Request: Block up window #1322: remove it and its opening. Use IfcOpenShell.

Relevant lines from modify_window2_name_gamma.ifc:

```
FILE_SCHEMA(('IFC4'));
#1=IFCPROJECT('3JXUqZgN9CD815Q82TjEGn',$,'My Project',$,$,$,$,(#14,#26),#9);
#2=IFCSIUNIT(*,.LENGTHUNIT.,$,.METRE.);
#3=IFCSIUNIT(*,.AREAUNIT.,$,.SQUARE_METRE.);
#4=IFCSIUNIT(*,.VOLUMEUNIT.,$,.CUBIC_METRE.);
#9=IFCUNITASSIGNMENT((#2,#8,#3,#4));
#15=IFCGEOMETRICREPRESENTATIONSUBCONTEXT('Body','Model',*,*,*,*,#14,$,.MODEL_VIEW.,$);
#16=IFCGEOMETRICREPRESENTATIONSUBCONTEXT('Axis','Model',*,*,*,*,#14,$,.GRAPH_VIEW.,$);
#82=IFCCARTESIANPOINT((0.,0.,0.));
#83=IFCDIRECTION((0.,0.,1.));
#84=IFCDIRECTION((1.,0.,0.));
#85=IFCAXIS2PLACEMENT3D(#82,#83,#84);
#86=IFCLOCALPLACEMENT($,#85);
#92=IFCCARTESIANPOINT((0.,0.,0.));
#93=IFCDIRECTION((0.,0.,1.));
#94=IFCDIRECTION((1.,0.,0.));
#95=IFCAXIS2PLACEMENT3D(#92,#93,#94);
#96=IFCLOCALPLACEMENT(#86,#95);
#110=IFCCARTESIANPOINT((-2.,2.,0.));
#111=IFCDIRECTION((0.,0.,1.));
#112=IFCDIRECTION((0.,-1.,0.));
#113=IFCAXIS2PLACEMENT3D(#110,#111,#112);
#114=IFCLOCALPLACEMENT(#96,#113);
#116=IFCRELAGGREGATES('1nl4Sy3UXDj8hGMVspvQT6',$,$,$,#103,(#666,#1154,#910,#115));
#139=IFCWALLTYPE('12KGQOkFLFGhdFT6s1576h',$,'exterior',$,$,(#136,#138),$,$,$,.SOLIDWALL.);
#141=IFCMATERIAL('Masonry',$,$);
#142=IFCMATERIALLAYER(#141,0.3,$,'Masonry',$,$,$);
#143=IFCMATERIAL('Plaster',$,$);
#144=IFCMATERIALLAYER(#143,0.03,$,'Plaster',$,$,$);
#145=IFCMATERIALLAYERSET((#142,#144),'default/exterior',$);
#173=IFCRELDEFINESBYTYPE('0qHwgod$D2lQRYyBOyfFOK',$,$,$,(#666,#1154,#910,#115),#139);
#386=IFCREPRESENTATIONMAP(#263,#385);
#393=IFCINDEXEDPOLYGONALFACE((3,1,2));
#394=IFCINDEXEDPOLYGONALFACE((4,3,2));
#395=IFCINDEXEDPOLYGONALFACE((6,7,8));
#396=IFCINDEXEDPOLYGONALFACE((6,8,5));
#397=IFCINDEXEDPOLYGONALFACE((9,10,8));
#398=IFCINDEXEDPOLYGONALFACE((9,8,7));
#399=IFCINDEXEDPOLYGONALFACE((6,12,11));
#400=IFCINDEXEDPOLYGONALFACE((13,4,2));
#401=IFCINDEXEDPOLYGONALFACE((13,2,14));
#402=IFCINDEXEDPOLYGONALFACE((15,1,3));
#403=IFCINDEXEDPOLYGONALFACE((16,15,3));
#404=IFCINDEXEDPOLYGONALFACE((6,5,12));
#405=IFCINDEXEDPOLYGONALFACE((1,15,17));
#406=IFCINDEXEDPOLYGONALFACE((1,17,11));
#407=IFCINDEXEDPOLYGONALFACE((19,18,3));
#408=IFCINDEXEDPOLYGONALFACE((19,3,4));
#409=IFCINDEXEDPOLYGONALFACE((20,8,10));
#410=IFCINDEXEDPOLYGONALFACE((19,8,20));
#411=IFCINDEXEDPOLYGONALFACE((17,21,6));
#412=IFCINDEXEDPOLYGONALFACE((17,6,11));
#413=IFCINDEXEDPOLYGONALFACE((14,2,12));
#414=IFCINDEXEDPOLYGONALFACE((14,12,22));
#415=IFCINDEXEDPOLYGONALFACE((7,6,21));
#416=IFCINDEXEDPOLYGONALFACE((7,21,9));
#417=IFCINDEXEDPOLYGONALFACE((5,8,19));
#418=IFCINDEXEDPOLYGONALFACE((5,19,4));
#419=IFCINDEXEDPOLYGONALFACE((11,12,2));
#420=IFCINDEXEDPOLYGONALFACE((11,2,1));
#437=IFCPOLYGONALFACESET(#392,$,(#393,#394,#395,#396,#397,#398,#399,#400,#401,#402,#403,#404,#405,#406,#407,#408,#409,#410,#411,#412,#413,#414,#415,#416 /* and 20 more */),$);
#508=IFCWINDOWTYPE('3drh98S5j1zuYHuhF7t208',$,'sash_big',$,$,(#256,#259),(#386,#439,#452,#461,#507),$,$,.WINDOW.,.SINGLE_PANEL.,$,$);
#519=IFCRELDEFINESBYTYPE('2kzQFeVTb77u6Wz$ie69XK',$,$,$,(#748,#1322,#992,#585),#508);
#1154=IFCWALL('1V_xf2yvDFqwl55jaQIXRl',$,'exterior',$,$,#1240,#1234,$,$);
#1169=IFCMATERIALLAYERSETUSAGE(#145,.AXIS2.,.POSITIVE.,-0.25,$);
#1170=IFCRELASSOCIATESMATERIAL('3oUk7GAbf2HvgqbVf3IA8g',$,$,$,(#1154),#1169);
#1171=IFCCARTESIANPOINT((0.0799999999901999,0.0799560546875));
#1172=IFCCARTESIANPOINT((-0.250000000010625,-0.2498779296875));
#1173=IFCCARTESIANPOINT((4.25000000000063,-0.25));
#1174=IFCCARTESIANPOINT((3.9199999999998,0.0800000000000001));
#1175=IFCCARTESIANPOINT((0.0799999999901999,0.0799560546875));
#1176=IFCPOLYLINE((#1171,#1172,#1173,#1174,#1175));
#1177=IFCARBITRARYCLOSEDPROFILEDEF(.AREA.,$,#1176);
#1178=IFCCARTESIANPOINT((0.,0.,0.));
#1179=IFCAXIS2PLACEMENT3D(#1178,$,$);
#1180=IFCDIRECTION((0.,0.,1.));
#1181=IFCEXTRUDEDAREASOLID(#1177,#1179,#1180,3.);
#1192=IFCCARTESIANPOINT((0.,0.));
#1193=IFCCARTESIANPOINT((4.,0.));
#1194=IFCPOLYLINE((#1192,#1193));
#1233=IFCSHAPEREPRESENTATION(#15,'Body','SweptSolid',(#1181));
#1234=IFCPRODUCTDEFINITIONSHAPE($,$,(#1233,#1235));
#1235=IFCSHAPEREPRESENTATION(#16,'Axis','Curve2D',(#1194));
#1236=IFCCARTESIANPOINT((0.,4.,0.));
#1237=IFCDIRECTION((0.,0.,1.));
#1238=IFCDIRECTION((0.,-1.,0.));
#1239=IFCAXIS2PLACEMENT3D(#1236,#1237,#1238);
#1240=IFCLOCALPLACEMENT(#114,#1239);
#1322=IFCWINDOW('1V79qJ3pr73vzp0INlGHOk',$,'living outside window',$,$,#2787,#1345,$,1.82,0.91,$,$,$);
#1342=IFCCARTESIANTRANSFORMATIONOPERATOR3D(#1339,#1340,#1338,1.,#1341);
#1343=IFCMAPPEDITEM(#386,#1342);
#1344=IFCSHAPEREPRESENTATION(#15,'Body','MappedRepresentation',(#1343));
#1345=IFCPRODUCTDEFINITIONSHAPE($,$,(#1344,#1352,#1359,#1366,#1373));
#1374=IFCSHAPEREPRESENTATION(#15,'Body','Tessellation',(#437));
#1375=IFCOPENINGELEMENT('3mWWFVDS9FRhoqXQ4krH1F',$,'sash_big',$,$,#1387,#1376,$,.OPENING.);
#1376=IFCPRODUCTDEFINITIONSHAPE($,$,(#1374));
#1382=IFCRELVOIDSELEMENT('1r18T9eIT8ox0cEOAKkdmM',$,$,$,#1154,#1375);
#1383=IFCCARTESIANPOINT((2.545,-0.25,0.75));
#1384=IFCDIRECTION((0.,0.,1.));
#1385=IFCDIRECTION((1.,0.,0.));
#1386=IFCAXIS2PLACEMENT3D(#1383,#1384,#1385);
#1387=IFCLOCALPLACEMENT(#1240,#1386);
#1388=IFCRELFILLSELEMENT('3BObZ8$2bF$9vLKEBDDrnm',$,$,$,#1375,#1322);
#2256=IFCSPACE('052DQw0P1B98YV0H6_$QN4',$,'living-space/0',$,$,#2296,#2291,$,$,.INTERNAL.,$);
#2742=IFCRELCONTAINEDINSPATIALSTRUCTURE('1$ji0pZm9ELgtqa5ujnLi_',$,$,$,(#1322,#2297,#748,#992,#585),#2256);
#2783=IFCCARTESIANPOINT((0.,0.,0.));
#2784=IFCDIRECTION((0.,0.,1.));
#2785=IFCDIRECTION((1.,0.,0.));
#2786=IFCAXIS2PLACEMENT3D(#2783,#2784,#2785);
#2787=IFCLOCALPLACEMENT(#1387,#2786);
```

```python
import ifcopenshell
import ifcopenshell.api.feature
import ifcopenshell.api.root
import ifcopenshell.geom
import ifcopenshell.util.shape

model = ifcopenshell.open("modify_window2_name_gamma.ifc")
settings = ifcopenshell.geom.settings()


def volume(element):
    """Net volume in cubic metres, openings subtracted."""
    shape = ifcopenshell.geom.create_shape(settings, element)
    return ifcopenshell.util.shape.get_volume(shape.geometry)


window = model.by_guid("1V79qJ3pr73vzp0INlGHOk")
opening = window.FillsVoids[0].RelatingOpeningElement
wall = opening.VoidsElements[0].RelatingBuildingElement
before = volume(wall)

ifcopenshell.api.root.remove_product(model, product=window)
ifcopenshell.api.feature.remove_feature(model, feature=opening)

after = volume(wall)

print(f"wall volume {before:.3f} -> {after:.3f} m3")

model.write("modify_window2_name_gamma_v2.ifc")
```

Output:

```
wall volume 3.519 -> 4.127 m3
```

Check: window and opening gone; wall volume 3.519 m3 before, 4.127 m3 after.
